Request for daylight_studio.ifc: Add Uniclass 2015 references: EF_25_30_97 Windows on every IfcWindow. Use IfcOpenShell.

First a look at what the model holds.

```python
import ifcopenshell

model = ifcopenshell.open("daylight_studio.ifc")
print(model.schema)
print("classifications:", [c.Name for c in model.by_type("IfcClassification")])
for ifc_class in ("IfcDoor", "IfcRoof", "IfcStair", "IfcWall", "IfcWindow"):
    print(ifc_class, len(model.by_type(ifc_class)))
```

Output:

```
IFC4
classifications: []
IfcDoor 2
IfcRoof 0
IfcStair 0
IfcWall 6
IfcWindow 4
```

```python
import ifcopenshell
import ifcopenshell.api.classification

model = ifcopenshell.open("daylight_studio.ifc")

system = ifcopenshell.api.classification.add_classification(model, classification="Uniclass 2015")

codes = {
    "IfcWindow": ("EF_25_30_97", "Windows"),
}
for ifc_class, (code, name) in codes.items():
    products = model.by_type(ifc_class)
    ifcopenshell.api.classification.add_reference(
        model, products=products, classification=system, identification=code, name=name
    )
    print(code, len(products))

model.write("daylight_studio_v2.ifc")
```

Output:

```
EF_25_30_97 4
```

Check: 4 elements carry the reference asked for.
